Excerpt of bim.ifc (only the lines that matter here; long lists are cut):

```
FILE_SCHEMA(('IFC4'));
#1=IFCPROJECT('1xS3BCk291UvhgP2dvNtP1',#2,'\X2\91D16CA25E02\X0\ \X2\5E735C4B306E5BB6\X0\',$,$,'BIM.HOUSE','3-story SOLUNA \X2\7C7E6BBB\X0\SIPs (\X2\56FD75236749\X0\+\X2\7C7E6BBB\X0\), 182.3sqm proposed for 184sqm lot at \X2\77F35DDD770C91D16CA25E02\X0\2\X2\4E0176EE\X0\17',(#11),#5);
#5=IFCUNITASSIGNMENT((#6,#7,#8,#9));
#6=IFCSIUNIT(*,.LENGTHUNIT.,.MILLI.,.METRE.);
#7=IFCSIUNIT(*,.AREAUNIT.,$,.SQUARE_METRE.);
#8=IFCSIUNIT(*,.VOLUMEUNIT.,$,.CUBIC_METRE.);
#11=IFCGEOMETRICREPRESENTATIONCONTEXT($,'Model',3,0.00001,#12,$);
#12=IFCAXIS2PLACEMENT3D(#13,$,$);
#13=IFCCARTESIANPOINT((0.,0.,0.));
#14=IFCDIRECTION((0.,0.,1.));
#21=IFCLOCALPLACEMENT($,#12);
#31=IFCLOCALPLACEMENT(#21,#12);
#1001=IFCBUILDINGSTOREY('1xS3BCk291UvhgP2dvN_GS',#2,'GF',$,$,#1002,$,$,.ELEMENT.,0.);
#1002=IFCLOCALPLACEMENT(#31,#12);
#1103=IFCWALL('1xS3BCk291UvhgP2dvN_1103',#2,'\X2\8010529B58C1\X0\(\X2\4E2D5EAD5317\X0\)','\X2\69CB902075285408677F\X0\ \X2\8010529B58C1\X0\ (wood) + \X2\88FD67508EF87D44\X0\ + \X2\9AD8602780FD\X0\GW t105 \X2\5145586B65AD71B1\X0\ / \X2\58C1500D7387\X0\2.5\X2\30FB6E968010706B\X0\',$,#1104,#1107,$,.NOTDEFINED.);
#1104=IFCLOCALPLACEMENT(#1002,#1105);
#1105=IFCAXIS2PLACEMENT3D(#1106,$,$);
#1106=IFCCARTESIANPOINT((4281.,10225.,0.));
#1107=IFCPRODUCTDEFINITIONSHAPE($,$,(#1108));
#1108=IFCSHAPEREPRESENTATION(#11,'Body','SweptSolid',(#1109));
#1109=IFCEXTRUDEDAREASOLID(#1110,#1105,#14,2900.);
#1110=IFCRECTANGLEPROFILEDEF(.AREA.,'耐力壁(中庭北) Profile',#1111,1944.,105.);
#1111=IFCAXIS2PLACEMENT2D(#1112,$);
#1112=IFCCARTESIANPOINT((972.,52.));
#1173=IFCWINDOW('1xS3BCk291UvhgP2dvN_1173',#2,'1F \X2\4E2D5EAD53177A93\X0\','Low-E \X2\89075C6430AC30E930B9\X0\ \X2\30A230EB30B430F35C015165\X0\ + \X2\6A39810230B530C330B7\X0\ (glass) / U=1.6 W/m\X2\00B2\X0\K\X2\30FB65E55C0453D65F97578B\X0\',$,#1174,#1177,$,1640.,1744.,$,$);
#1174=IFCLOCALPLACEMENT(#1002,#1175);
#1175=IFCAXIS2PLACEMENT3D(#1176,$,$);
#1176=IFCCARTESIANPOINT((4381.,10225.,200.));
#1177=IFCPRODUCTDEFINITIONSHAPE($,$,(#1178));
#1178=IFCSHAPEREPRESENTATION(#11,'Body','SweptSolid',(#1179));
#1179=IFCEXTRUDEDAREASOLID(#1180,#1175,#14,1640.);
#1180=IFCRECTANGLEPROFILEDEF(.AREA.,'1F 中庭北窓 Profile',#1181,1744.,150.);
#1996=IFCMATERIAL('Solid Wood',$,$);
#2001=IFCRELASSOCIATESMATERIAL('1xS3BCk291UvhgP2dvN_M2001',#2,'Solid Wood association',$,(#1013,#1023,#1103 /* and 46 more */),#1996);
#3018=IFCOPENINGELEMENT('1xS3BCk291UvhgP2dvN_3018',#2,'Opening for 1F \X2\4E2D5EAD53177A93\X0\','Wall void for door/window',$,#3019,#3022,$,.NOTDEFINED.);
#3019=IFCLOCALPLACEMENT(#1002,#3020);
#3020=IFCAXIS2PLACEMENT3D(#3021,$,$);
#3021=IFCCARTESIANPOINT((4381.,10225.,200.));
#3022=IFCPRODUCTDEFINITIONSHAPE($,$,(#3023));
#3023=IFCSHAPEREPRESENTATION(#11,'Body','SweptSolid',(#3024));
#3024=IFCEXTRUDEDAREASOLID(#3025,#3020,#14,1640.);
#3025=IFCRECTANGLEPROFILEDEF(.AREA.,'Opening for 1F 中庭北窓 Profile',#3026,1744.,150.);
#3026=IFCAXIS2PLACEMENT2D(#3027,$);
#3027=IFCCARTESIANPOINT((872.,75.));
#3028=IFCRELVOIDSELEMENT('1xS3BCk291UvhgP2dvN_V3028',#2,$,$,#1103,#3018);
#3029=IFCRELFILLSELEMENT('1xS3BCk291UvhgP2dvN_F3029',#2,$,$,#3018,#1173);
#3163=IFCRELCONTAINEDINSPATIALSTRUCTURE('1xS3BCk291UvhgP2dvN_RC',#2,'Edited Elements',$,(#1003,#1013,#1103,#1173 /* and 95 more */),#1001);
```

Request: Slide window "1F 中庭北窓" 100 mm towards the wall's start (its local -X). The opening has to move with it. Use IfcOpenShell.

```python
import ifcopenshell
import ifcopenshell.api.geometry
import ifcopenshell.util.placement
import ifcopenshell.util.unit

model = ifcopenshell.open("bim.ifc")
unit_scale = ifcopenshell.util.unit.calculate_unit_scale(model)

window = model.by_id(1173)
opening = window.FillsVoids[0].RelatingOpeningElement
wall = opening.VoidsElements[0].RelatingBuildingElement

wall_matrix = ifcopenshell.util.placement.get_local_placement(wall.ObjectPlacement)
shift = wall_matrix[:3, 0] * -0.1 / unit_scale
before = ifcopenshell.util.placement.get_local_placement(window.ObjectPlacement)[:3, 3].copy()

# The window is not placed relative to its opening, so move both.
for product in (opening, window):
    matrix = ifcopenshell.util.placement.get_local_placement(product.ObjectPlacement)
    matrix[:3, 3] += shift
    ifcopenshell.api.geometry.edit_object_placement(model, product=product, matrix=matrix, is_si=False)

after = ifcopenshell.util.placement.get_local_placement(window.ObjectPlacement)[:3, 3]
print("window moved by", (after - before).round(3) + 0.0)

model.write("bim_edited.ifc")
```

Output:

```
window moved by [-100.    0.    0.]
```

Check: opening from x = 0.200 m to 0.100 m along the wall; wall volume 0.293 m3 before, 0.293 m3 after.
